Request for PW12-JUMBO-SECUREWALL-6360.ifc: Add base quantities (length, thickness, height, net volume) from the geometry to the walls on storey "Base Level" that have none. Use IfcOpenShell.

First a look at what the model holds.

```python
import ifcopenshell
import ifcopenshell.util.element
import ifcopenshell.util.unit

model = ifcopenshell.open("PW12-JUMBO-SECUREWALL-6360.ifc")
print(model.schema)
for unit_type in ("LENGTHUNIT", "AREAUNIT", "VOLUMEUNIT"):
    print(unit_type, ifcopenshell.util.unit.calculate_unit_scale(model, unit_type))
storey = next(s for s in model.by_type("IfcBuildingStorey") if s.Name == "Base Level")
walls = [e for e in ifcopenshell.util.element.get_decomposition(storey) if e.is_a("IfcWall")]
for e in sorted(walls, key=lambda e: e.id()):
    print(e.id(), e.is_a(), e.Name, list(ifcopenshell.util.element.get_psets(e, qtos_only=True)), sep=" | ")
```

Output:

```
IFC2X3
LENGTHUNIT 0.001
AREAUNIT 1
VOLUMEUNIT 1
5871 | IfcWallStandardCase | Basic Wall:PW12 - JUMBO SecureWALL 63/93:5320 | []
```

```python
import ifcopenshell
import ifcopenshell.api.pset
import ifcopenshell.geom
import ifcopenshell.util.element
import ifcopenshell.util.shape
import ifcopenshell.util.unit

model = ifcopenshell.open("PW12-JUMBO-SECUREWALL-6360.ifc")
unit_scale = ifcopenshell.util.unit.calculate_unit_scale(model)
volume_scale = ifcopenshell.util.unit.calculate_unit_scale(model, "VOLUMEUNIT")
settings = ifcopenshell.geom.settings()

storey = next(s for s in model.by_type("IfcBuildingStorey") if s.Name == "Base Level")
walls = [e for e in ifcopenshell.util.element.get_decomposition(storey) if e.is_a("IfcWall")]

for e in sorted(walls, key=lambda e: e.id()):
    if ifcopenshell.util.element.get_psets(e, qtos_only=True, should_inherit=False):
        continue
    # Geometry comes back in metres, in the element's own axes.
    shape = ifcopenshell.geom.create_shape(settings, e)
    values = {
        "Length": ifcopenshell.util.shape.get_x(shape.geometry) / unit_scale,
        "Width": ifcopenshell.util.shape.get_y(shape.geometry) / unit_scale,
        "Height": ifcopenshell.util.shape.get_z(shape.geometry) / unit_scale,
        "NetVolume": ifcopenshell.util.shape.get_volume(shape.geometry) / volume_scale,
    }
    qto = ifcopenshell.api.pset.add_qto(model, product=e, name="BaseQuantities")
    ifcopenshell.api.pset.edit_qto(model, qto=qto, properties=values)
    print(e.id(), {k: round(v, 3) for k, v in values.items()})

model.write("PW12-JUMBO-SECUREWALL-6360_edited.ifc")
```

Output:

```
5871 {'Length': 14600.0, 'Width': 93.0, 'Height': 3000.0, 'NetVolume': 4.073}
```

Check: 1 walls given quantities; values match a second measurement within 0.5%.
